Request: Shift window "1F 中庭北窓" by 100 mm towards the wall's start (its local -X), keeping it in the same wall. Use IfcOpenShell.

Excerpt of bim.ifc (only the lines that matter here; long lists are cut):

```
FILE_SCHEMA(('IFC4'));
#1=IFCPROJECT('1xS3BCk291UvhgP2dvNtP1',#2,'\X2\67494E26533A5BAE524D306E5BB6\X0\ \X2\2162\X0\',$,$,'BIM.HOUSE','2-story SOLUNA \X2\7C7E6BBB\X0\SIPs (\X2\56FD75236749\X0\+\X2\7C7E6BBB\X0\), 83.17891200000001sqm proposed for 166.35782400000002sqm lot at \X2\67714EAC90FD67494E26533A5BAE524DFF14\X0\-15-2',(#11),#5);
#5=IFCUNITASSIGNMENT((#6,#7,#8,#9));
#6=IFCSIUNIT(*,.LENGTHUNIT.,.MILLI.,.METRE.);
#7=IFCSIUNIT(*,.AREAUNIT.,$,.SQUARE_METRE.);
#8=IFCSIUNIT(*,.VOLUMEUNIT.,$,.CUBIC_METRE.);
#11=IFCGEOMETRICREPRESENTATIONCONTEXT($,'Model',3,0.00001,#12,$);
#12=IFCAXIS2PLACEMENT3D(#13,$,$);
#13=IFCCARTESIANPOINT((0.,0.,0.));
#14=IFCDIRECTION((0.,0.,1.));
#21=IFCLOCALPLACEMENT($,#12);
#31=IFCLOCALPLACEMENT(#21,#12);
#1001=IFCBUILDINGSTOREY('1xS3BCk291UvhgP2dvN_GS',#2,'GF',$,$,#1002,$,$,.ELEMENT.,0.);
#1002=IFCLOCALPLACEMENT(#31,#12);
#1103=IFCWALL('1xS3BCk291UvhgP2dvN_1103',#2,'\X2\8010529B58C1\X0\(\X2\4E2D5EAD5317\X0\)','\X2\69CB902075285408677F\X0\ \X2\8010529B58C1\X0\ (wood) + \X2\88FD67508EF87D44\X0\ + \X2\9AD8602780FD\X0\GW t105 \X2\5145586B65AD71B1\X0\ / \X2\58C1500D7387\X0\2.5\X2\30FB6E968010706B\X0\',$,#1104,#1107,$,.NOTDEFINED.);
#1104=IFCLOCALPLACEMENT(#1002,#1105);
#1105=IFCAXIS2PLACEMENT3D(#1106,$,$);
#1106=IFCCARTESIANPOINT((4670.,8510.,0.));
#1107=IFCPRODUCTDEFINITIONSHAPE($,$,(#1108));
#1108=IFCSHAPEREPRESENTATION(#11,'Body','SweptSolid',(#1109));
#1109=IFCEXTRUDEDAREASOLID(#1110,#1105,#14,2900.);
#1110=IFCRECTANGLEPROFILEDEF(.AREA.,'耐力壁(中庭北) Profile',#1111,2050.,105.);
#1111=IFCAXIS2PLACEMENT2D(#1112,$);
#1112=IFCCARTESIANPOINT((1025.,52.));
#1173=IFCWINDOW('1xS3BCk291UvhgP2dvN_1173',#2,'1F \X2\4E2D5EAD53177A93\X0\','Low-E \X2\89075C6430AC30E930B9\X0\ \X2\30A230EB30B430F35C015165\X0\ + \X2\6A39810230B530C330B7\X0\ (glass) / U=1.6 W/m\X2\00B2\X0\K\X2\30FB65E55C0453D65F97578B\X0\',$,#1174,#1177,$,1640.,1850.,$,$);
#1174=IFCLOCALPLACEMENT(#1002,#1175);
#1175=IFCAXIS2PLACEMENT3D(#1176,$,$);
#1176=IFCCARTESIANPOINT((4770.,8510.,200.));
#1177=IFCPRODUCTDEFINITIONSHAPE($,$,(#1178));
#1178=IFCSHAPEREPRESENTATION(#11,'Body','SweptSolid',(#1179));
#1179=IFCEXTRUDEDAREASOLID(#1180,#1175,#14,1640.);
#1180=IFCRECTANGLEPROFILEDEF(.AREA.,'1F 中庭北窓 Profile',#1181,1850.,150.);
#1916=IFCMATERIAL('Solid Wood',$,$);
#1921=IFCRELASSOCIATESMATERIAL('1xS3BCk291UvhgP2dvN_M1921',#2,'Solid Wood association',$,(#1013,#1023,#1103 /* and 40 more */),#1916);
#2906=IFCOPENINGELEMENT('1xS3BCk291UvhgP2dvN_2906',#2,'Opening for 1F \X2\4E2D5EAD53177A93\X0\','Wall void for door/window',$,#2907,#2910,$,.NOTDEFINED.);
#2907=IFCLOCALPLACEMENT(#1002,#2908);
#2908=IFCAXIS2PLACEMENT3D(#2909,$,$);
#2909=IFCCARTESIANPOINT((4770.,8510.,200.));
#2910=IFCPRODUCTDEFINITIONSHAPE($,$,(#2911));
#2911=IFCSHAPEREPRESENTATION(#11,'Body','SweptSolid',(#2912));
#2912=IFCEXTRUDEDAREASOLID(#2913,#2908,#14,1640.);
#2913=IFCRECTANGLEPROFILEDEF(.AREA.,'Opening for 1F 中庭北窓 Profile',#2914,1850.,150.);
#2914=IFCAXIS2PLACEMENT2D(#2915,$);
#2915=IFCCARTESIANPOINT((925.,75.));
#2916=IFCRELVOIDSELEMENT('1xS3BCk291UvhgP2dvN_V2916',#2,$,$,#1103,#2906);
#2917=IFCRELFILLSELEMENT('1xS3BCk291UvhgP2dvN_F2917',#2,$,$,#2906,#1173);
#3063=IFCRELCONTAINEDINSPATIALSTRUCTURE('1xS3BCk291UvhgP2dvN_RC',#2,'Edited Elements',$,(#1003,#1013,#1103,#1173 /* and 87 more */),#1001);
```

```python
import ifcopenshell
import ifcopenshell.api.geometry
import ifcopenshell.util.placement
import ifcopenshell.util.unit

model = ifcopenshell.open("bim.ifc")
unit_scale = ifcopenshell.util.unit.calculate_unit_scale(model)

window = model.by_guid("1xS3BCk291UvhgP2dvN_1173")
opening = window.FillsVoids[0].RelatingOpeningElement
wall = opening.VoidsElements[0].RelatingBuildingElement

wall_matrix = ifcopenshell.util.placement.get_local_placement(wall.ObjectPlacement)
shift = wall_matrix[:3, 0] * -0.1 / unit_scale
before = ifcopenshell.util.placement.get_local_placement(window.ObjectPlacement)[:3, 3].copy()

# The window is not placed relative to its opening, so move both.
for product in (opening, window):
    matrix = ifcopenshell.util.placement.get_local_placement(product.ObjectPlacement)
    matrix[:3, 3] += shift
    ifcopenshell.api.geometry.edit_object_placement(model, product=product, matrix=matrix, is_si=False)

after = ifcopenshell.util.placement.get_local_placement(window.ObjectPlacement)[:3, 3]
print("window moved by", (after - before).round(3) + 0.0)

model.write("bim_v2.ifc")
```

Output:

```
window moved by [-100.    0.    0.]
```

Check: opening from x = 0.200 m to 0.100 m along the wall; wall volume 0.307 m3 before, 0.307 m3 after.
